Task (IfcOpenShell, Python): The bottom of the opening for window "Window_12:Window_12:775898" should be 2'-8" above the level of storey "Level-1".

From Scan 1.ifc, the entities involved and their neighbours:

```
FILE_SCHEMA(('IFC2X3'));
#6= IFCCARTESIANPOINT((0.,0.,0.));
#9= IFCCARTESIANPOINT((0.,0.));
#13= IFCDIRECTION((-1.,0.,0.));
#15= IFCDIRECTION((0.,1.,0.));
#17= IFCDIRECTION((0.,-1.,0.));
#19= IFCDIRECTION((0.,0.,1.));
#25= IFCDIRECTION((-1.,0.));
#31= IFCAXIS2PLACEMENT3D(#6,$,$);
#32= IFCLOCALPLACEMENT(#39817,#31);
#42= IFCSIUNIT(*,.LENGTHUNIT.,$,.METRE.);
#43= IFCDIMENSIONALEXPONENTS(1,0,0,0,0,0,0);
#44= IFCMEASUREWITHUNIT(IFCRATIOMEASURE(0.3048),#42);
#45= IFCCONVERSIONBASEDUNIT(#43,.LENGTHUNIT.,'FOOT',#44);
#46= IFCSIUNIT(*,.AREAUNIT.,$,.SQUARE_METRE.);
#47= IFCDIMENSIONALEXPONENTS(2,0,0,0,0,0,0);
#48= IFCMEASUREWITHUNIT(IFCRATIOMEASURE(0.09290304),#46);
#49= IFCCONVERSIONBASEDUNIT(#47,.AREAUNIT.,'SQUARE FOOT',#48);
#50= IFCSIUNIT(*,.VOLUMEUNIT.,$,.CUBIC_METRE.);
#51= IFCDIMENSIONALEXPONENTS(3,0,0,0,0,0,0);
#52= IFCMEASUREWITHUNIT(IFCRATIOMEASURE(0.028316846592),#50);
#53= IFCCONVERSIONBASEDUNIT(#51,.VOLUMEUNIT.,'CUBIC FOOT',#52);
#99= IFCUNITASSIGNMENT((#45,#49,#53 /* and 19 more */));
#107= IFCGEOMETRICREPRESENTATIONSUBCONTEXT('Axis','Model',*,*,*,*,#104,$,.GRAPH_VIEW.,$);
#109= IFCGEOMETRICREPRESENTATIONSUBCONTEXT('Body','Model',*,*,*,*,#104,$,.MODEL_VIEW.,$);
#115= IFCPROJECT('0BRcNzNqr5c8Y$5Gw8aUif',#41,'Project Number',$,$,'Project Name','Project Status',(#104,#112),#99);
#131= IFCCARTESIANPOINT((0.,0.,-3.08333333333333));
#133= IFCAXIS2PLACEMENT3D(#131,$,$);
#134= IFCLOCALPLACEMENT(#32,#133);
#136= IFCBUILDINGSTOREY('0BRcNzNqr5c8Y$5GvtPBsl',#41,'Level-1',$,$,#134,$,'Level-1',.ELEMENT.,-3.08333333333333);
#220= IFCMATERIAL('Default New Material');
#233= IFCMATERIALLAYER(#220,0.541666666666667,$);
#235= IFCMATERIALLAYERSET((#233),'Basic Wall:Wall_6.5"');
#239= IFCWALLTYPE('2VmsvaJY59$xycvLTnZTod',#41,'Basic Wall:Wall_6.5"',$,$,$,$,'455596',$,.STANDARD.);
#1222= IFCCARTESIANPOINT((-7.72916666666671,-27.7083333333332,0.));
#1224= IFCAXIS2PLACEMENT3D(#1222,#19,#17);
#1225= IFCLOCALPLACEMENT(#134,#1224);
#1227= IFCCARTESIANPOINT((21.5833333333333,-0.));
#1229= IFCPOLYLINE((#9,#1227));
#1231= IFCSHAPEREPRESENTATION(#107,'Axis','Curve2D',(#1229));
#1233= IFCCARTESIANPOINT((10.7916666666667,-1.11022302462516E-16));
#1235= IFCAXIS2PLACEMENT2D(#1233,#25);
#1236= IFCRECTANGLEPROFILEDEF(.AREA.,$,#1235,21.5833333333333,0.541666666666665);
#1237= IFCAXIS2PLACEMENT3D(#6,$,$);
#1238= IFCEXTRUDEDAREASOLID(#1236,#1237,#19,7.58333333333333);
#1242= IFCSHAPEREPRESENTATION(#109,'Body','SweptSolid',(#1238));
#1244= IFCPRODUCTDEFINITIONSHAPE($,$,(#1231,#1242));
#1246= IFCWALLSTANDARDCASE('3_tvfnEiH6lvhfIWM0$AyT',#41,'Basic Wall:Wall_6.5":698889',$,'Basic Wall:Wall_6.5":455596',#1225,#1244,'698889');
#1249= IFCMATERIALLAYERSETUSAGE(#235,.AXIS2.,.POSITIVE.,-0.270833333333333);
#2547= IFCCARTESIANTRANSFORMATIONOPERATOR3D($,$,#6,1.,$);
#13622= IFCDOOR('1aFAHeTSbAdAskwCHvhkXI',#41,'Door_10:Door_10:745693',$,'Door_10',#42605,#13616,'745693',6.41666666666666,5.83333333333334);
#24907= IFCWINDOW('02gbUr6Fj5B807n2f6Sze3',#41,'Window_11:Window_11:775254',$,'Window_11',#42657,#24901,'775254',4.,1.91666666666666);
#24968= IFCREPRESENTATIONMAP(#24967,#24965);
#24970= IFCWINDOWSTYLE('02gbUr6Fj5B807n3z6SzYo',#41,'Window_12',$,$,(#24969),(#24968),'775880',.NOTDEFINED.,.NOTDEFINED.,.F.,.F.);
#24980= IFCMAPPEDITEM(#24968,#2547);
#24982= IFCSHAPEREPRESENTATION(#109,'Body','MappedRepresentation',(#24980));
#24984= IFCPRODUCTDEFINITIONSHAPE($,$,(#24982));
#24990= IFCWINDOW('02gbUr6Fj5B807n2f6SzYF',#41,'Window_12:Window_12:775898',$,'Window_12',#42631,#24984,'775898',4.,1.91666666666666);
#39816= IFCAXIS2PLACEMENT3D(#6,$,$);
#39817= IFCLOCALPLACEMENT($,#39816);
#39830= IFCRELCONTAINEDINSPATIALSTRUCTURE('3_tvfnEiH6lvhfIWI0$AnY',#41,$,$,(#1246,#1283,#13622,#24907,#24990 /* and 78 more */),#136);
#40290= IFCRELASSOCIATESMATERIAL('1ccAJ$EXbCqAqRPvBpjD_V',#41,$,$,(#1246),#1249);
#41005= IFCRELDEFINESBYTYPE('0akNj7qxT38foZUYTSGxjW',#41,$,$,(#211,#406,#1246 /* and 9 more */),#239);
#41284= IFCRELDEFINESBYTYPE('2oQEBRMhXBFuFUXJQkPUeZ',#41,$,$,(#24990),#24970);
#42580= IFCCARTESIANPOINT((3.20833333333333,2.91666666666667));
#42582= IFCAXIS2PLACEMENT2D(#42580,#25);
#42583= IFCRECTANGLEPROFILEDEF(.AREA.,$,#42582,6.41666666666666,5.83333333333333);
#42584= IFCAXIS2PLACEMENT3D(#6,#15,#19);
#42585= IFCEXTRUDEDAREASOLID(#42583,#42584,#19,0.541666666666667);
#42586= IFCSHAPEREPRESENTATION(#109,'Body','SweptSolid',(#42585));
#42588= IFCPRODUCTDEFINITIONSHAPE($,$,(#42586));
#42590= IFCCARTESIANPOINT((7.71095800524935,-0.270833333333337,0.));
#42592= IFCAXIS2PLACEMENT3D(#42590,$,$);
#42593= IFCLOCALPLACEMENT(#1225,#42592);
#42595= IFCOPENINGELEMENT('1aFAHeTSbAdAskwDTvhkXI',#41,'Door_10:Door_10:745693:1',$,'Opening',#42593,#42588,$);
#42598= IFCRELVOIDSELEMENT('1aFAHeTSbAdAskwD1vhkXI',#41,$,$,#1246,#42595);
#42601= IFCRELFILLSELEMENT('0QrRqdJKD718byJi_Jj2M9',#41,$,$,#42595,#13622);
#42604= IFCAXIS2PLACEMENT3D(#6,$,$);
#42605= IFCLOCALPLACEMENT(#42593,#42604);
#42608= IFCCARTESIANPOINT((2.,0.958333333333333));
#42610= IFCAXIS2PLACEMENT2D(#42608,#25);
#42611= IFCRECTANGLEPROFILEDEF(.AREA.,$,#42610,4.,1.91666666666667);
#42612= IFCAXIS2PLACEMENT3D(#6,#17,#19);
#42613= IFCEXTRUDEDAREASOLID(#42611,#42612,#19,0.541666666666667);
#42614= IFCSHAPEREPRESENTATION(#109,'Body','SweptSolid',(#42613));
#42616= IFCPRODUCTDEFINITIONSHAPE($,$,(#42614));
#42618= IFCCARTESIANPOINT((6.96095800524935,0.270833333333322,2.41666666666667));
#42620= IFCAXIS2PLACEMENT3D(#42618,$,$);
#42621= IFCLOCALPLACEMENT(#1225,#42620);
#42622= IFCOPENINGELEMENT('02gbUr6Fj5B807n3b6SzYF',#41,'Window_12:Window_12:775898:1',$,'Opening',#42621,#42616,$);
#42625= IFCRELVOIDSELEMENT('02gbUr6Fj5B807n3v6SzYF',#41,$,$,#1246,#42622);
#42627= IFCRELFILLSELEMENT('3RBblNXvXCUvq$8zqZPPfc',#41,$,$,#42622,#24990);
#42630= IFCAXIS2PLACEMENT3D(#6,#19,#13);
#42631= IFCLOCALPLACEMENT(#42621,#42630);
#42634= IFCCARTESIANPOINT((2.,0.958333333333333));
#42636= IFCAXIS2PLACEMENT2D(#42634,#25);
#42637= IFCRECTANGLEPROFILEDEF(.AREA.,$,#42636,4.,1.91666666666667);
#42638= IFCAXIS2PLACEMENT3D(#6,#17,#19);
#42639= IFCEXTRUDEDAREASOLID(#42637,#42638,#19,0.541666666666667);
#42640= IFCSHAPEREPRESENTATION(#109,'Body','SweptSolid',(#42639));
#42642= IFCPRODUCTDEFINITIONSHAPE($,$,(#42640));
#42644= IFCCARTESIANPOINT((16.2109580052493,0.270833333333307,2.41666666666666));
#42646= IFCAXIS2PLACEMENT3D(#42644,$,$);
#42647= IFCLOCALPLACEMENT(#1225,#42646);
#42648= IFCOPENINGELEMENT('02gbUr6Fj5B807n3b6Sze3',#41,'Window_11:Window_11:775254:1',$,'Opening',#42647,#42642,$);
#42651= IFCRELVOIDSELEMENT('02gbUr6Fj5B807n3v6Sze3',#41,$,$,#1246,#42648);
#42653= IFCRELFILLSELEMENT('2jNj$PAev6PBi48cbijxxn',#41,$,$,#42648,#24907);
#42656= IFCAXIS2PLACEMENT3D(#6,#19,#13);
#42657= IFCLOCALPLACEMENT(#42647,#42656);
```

```python
import numpy as np
import ifcopenshell
import ifcopenshell.api.geometry
import ifcopenshell.geom
import ifcopenshell.util.element
import ifcopenshell.util.placement
import ifcopenshell.util.shape
import ifcopenshell.util.unit

model = ifcopenshell.open("Scan 1.ifc")
unit_scale = ifcopenshell.util.unit.calculate_unit_scale(model)

window = model.by_guid("02gbUr6Fj5B807n2f6SzYF")
opening = window.FillsVoids[0].RelatingOpeningElement
storey = ifcopenshell.util.element.get_container(window, ifc_class="IfcBuildingStorey")
level = ifcopenshell.util.placement.get_local_placement(storey.ObjectPlacement)[2, 3]

# The opening's origin need not be at the sill, so measure its lowest point.
shape = ifcopenshell.geom.create_shape(ifcopenshell.geom.settings(), opening)
bottom = ifcopenshell.util.shape.get_shape_bottom_elevation(shape, shape.geometry) / unit_scale
dz = level + 32 * 0.0254 / unit_scale - bottom

shift = np.array([0.0, 0.0, dz])
# The window is placed relative to its opening, so it follows when the opening moves.
matrix = ifcopenshell.util.placement.get_local_placement(opening.ObjectPlacement)
matrix[:3, 3] += shift
ifcopenshell.api.geometry.edit_object_placement(
    model, product=opening, matrix=matrix, is_si=False, should_transform_children=True
)

print(f"moved by {dz * unit_scale:+.3f} m")

model.write("Scan 1_v2.ifc")
```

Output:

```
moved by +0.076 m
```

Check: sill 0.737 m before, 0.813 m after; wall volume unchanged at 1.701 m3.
